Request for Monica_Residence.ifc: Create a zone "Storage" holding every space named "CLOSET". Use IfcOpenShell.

First a look at what the model holds.

```python
import ifcopenshell

model = ifcopenshell.open("Monica_Residence.ifc")
print(model.schema)
seen = {}
for space in model.by_type("IfcSpace"):
    seen[space.LongName] = seen.get(space.LongName, 0) + 1
for name, count in sorted(seen.items(), key=str):
    print(count, "x", name)
print("zones:", [z.Name for z in model.by_type("IfcZone")][:20])
```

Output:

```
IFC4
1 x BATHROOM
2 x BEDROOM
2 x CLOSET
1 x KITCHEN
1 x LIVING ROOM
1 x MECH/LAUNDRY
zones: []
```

```python
import ifcopenshell
import ifcopenshell.api.group
import ifcopenshell.api.root

model = ifcopenshell.open("Monica_Residence.ifc")

names = {"CLOSET"}
spaces = [s for s in model.by_type("IfcSpace") if s.LongName in names]

zone = ifcopenshell.api.root.create_entity(model, ifc_class="IfcZone", name="Storage")
ifcopenshell.api.group.assign_group(model, products=spaces, group=zone)
print(len(spaces), "spaces in", zone.Name)

model.write("Monica_Residence-out.ifc")
```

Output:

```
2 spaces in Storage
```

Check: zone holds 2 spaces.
